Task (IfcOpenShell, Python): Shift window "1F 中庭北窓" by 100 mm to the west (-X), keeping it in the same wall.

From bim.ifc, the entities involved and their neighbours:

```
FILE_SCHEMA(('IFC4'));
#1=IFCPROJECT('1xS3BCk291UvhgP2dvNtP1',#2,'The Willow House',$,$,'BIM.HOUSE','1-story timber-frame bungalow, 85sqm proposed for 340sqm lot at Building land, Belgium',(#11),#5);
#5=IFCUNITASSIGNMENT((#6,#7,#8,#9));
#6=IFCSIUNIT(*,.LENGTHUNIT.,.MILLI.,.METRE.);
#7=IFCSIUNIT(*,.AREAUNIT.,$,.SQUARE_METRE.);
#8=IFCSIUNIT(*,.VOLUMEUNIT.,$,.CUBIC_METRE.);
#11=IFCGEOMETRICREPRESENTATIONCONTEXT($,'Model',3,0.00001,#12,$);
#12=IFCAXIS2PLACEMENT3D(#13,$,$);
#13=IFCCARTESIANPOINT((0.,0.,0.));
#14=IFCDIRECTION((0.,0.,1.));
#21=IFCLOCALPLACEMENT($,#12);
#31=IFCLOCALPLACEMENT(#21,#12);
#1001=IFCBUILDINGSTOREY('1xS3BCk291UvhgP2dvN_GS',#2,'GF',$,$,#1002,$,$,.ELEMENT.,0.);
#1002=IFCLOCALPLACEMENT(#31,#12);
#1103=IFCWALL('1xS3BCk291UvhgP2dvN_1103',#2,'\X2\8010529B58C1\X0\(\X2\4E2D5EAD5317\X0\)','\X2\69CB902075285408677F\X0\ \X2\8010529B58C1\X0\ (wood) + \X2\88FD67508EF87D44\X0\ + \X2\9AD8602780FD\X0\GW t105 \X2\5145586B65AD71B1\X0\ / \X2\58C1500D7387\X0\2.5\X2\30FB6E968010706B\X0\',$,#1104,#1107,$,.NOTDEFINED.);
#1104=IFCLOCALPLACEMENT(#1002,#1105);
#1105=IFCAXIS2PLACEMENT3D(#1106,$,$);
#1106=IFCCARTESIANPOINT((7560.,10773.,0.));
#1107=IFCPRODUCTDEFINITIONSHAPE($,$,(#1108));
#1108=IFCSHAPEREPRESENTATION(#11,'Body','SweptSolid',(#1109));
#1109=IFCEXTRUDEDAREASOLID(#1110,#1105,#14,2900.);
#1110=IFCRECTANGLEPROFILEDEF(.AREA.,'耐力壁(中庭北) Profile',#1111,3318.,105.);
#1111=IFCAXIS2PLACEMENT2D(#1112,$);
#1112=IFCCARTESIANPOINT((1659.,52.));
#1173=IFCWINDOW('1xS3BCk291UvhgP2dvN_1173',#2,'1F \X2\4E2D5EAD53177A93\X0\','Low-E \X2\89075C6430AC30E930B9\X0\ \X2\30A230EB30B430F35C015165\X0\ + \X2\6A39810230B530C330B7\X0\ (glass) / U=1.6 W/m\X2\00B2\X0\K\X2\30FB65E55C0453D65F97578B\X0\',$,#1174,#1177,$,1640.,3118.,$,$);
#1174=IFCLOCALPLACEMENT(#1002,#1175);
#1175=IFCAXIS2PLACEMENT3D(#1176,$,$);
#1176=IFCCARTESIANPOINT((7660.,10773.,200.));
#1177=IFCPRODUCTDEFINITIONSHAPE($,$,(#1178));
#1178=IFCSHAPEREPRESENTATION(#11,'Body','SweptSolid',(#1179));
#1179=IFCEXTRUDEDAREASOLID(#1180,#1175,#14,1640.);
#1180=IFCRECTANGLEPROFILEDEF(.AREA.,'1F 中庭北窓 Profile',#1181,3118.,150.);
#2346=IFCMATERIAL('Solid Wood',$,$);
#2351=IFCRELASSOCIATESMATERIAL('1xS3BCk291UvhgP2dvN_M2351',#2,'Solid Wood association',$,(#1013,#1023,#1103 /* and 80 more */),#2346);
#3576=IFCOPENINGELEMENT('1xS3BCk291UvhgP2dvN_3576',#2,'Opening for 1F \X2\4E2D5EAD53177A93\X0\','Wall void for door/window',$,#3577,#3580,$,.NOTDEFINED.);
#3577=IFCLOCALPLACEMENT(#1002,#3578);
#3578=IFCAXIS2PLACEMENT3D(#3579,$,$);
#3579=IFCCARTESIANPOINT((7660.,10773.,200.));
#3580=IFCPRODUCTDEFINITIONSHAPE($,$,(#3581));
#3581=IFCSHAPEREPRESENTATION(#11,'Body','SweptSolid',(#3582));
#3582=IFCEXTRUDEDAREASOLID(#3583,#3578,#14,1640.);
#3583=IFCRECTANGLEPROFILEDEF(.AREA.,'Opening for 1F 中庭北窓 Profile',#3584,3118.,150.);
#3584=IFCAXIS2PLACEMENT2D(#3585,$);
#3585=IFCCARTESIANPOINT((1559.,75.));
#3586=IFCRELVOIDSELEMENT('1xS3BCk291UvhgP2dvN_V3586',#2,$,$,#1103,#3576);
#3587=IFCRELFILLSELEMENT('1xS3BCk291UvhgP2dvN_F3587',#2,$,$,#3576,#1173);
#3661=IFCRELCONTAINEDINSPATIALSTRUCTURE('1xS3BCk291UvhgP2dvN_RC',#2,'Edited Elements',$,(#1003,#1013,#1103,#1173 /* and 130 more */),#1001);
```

```python
import ifcopenshell
import ifcopenshell.api.geometry
import ifcopenshell.util.placement
import ifcopenshell.util.unit

model = ifcopenshell.open("bim.ifc")
unit_scale = ifcopenshell.util.unit.calculate_unit_scale(model)

window = model.by_id(1173)
opening = window.FillsVoids[0].RelatingOpeningElement
wall = opening.VoidsElements[0].RelatingBuildingElement

wall_matrix = ifcopenshell.util.placement.get_local_placement(wall.ObjectPlacement)
shift = wall_matrix[:3, 0] * -0.1 / unit_scale
before = ifcopenshell.util.placement.get_local_placement(window.ObjectPlacement)[:3, 3].copy()

# The window is not placed relative to its opening, so move both.
for product in (opening, window):
    matrix = ifcopenshell.util.placement.get_local_placement(product.ObjectPlacement)
    matrix[:3, 3] += shift
    ifcopenshell.api.geometry.edit_object_placement(model, product=product, matrix=matrix, is_si=False)

after = ifcopenshell.util.placement.get_local_placement(window.ObjectPlacement)[:3, 3]
print("window moved by", (after - before).round(3) + 0.0)

model.write("bim-out.ifc")
```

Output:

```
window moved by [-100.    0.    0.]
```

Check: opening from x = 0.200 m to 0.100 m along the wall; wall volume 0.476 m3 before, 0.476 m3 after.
